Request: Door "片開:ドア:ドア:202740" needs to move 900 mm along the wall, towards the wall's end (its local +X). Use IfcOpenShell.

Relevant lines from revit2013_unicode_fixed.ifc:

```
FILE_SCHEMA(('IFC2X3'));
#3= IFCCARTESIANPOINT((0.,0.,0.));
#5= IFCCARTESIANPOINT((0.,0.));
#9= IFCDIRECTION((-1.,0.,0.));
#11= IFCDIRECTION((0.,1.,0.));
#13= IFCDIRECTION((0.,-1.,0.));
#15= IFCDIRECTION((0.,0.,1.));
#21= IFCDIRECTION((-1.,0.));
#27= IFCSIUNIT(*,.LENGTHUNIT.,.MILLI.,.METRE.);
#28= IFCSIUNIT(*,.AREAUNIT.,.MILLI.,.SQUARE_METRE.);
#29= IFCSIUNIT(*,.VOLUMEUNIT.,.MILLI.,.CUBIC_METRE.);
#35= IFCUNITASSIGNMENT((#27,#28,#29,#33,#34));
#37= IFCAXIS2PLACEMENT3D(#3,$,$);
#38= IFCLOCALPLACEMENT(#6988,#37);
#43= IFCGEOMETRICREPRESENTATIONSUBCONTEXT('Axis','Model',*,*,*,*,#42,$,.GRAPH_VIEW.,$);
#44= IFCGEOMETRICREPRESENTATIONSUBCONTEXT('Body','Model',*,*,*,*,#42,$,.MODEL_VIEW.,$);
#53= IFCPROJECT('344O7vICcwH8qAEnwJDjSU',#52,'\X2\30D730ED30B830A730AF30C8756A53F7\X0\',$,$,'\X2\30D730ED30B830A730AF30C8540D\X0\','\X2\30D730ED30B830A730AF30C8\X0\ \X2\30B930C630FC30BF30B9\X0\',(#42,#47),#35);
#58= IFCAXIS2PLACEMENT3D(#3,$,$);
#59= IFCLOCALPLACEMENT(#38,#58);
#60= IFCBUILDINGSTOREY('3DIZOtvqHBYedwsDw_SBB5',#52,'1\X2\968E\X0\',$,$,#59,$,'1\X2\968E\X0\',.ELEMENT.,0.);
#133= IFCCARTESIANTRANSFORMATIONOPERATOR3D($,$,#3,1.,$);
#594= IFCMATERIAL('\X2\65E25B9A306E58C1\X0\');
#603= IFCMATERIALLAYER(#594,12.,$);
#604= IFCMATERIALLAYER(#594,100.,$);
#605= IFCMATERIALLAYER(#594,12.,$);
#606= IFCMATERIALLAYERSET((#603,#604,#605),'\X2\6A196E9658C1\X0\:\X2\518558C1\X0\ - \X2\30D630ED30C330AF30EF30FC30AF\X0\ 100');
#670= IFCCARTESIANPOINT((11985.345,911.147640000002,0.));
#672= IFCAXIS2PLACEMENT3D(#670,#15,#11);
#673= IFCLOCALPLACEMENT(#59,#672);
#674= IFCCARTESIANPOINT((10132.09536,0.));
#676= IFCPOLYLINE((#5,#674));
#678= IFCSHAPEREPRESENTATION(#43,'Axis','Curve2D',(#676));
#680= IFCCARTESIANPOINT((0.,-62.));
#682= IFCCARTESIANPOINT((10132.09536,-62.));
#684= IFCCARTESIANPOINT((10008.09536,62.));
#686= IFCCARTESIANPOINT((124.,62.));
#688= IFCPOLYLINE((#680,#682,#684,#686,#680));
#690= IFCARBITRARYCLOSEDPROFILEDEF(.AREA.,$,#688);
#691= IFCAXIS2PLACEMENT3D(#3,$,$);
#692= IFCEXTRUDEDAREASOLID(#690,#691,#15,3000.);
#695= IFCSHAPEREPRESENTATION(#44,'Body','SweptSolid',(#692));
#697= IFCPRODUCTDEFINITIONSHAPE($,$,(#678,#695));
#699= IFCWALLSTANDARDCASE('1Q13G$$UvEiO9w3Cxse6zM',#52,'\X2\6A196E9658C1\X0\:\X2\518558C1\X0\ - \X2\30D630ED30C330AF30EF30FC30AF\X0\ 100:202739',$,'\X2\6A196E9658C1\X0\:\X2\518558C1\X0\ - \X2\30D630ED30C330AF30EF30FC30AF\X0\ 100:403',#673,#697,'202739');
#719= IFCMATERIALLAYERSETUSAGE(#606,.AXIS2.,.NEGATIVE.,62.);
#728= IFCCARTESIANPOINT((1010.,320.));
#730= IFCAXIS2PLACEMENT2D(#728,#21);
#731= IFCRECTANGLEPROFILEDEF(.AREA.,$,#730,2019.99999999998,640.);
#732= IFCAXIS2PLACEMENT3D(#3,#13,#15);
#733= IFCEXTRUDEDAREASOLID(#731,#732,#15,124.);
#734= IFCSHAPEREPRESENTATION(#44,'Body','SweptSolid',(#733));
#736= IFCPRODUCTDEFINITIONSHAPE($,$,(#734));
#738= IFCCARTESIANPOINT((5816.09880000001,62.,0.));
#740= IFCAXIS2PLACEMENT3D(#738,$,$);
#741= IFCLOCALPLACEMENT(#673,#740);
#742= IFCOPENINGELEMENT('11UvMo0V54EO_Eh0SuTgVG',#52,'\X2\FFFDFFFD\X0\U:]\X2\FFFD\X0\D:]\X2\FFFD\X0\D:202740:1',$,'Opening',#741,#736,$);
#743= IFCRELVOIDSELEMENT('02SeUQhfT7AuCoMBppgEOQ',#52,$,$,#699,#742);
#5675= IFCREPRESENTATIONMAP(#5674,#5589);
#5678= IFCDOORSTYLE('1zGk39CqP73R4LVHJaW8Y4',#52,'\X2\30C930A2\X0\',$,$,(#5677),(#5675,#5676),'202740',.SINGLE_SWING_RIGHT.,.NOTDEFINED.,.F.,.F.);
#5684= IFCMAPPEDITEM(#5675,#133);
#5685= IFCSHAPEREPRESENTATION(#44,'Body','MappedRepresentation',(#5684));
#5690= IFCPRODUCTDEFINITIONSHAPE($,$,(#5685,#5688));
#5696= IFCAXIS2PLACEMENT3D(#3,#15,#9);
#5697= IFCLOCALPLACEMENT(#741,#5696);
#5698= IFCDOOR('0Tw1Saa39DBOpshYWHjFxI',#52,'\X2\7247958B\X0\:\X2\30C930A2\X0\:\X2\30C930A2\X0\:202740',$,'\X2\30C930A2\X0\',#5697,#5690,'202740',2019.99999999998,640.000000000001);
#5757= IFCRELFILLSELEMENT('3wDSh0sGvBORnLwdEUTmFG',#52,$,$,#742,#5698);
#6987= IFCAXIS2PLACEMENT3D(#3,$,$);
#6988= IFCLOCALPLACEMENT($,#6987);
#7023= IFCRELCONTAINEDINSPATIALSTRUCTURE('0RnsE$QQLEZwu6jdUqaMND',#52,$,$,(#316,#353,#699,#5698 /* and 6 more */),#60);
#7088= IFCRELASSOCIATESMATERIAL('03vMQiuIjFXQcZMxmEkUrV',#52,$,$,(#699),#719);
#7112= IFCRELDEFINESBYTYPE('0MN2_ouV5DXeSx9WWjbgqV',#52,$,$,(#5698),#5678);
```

```python
import ifcopenshell
import ifcopenshell.api.geometry
import ifcopenshell.util.placement

model = ifcopenshell.open("revit2013_unicode_fixed.ifc")

door = model.by_guid("0Tw1Saa39DBOpshYWHjFxI")
opening = door.FillsVoids[0].RelatingOpeningElement
wall = opening.VoidsElements[0].RelatingBuildingElement

wall_matrix = ifcopenshell.util.placement.get_local_placement(wall.ObjectPlacement)
shift = wall_matrix[:3, 0] * 900.0
before = ifcopenshell.util.placement.get_local_placement(door.ObjectPlacement)[:3, 3].copy()

# The door is placed relative to its opening, so it follows when the opening moves.
matrix = ifcopenshell.util.placement.get_local_placement(opening.ObjectPlacement)
matrix[:3, 3] += shift
ifcopenshell.api.geometry.edit_object_placement(
    model, product=opening, matrix=matrix, is_si=False, should_transform_children=True
)

after = ifcopenshell.util.placement.get_local_placement(door.ObjectPlacement)[:3, 3]
print("door moved by", (after - before).round(3) + 0.0)

model.write("revit2013_unicode_fixed_rev.ifc")
```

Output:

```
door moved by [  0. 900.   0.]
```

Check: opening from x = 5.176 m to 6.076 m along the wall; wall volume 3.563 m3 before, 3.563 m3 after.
